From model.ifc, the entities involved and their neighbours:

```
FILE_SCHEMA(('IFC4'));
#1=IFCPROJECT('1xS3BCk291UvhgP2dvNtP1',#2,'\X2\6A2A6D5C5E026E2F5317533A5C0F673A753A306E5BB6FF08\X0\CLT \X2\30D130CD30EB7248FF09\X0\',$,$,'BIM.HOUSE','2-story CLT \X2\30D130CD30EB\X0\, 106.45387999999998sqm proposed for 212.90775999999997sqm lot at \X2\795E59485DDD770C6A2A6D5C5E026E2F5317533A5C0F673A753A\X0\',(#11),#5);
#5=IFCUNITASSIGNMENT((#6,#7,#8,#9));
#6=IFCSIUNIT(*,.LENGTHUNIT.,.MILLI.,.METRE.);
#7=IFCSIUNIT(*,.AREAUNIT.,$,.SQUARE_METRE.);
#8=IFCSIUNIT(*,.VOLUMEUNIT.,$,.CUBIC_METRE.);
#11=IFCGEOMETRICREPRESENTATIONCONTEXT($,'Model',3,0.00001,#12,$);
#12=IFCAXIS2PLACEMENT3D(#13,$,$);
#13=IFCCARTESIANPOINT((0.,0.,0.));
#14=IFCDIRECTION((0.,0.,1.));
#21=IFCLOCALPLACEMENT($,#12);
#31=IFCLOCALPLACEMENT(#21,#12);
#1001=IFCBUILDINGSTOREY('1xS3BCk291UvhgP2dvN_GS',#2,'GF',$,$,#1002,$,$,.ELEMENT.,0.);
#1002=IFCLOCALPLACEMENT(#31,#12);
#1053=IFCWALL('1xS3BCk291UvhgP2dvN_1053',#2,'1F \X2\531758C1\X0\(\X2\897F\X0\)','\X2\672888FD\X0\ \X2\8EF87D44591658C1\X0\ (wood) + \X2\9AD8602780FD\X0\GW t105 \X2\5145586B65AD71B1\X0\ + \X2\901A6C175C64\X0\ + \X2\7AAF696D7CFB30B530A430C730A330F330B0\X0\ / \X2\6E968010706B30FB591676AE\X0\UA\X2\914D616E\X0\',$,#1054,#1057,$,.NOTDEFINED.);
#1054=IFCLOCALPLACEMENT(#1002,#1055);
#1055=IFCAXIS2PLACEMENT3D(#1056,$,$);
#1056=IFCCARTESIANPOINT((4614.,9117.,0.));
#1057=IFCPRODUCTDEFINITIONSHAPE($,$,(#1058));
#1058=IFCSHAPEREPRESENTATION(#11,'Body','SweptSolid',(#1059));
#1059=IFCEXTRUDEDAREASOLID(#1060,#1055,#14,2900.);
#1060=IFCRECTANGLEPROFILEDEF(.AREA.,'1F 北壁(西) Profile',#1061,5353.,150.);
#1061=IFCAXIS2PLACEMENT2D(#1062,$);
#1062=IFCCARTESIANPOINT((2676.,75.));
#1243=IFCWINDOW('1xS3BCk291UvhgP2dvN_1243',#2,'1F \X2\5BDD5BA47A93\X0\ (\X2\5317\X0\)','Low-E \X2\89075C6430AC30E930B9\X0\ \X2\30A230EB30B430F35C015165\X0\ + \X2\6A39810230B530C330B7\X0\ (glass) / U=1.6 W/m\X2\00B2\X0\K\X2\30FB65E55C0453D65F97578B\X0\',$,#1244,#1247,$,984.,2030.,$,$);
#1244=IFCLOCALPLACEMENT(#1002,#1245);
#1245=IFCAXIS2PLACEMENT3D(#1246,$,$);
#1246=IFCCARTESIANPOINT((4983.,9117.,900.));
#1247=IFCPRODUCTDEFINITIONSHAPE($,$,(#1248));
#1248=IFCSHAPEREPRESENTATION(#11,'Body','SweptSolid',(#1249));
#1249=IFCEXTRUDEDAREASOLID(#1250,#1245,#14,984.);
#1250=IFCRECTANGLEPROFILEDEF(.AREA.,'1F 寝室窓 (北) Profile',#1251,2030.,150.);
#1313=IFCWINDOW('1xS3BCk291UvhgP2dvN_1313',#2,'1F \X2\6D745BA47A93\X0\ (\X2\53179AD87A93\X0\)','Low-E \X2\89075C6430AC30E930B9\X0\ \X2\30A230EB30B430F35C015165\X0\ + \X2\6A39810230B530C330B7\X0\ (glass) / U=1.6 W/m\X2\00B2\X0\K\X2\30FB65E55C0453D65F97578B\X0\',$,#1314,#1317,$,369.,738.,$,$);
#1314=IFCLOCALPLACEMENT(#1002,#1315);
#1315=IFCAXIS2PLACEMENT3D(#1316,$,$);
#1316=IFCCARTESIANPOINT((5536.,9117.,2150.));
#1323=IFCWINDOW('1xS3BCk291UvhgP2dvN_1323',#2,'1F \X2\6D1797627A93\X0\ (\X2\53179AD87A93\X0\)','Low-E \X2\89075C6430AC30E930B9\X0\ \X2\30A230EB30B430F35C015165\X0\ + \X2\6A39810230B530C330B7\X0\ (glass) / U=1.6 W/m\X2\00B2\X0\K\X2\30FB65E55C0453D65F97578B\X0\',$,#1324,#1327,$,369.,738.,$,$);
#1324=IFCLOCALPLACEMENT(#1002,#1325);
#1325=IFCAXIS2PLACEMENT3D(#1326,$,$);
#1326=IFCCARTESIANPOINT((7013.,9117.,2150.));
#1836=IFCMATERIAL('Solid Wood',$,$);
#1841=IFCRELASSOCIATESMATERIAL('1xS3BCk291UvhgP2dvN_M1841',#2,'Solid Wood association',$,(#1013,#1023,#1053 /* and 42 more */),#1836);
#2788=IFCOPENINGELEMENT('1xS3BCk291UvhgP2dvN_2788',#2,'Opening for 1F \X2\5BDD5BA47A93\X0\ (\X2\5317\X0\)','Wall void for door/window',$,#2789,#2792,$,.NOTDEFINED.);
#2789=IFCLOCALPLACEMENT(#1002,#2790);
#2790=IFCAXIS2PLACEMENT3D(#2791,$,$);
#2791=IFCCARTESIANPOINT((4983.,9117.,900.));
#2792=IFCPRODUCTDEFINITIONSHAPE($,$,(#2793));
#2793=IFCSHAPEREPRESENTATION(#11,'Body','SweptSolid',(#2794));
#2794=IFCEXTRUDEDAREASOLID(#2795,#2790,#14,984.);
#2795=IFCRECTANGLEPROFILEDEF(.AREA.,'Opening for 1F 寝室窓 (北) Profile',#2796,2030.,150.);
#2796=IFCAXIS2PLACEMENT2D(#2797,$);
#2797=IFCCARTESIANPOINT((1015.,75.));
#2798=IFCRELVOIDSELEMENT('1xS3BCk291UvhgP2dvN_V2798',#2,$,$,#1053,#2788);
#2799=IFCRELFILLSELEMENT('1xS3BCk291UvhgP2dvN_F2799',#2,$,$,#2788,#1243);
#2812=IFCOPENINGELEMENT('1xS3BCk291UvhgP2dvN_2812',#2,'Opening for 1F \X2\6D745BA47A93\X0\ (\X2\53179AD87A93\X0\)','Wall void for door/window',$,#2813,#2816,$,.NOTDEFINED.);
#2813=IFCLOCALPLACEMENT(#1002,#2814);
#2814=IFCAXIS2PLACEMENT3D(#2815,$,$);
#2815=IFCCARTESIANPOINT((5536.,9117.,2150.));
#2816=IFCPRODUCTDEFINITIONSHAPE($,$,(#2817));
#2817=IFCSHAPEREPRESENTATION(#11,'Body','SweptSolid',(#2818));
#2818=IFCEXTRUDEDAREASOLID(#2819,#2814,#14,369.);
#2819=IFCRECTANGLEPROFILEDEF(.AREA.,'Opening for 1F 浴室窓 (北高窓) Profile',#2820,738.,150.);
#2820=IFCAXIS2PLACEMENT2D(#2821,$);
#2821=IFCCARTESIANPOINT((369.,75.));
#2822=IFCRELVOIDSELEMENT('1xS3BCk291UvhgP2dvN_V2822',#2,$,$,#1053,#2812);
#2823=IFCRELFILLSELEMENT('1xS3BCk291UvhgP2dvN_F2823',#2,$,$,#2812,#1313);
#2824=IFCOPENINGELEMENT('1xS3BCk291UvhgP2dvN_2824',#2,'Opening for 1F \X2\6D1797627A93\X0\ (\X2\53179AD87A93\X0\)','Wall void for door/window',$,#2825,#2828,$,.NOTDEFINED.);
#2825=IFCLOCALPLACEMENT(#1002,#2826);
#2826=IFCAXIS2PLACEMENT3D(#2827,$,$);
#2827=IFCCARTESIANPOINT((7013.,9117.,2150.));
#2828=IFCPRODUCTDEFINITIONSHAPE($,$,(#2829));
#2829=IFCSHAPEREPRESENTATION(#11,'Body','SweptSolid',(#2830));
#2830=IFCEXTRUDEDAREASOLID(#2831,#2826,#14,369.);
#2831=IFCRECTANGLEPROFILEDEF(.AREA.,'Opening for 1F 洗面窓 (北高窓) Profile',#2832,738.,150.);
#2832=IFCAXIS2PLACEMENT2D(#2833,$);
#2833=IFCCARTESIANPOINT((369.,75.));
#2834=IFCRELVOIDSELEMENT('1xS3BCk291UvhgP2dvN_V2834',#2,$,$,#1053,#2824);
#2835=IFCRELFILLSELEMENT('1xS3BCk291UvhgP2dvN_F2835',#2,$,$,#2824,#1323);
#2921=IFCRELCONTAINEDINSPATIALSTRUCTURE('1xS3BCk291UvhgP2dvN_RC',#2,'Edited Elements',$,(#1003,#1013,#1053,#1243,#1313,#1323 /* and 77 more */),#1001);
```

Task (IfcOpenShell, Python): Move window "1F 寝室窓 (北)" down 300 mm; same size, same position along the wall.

```python
import numpy as np
import ifcopenshell
import ifcopenshell.api.geometry
import ifcopenshell.util.placement
import ifcopenshell.util.unit

model = ifcopenshell.open("model.ifc")
unit_scale = ifcopenshell.util.unit.calculate_unit_scale(model)

window = model.by_guid("1xS3BCk291UvhgP2dvN_1243")
opening = window.FillsVoids[0].RelatingOpeningElement
dz = -0.3 / unit_scale

shift = np.array([0.0, 0.0, dz])
# The window is not placed relative to its opening, so move both.
for product in (opening, window):
    matrix = ifcopenshell.util.placement.get_local_placement(product.ObjectPlacement)
    matrix[:3, 3] += shift
    ifcopenshell.api.geometry.edit_object_placement(model, product=product, matrix=matrix, is_si=False)

print(f"moved by {dz * unit_scale:+.3f} m")

model.write("model_rev.ifc")
```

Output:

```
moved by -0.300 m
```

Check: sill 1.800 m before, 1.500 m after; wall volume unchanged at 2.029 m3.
